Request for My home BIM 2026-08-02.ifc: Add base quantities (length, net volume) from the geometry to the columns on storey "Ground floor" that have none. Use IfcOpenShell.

First a look at what the model holds.

```python
import ifcopenshell
import ifcopenshell.util.element
import ifcopenshell.util.unit

model = ifcopenshell.open("My home BIM 2026-08-02.ifc")
print(model.schema)
for unit_type in ("LENGTHUNIT", "AREAUNIT", "VOLUMEUNIT"):
    print(unit_type, ifcopenshell.util.unit.calculate_unit_scale(model, unit_type))
storey = next(s for s in model.by_type("IfcBuildingStorey") if s.Name == "Ground floor")
columns = [e for e in ifcopenshell.util.element.get_decomposition(storey) if e.is_a("IfcColumn")]
for e in sorted(columns, key=lambda e: e.id()):
    print(e.id(), e.is_a(), e.Name, list(ifcopenshell.util.element.get_psets(e, qtos_only=True)), sep=" | ")
```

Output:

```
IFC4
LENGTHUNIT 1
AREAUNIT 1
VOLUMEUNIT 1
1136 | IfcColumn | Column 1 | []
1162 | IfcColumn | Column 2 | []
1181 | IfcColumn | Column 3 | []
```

```python
import ifcopenshell
import ifcopenshell.api.pset
import ifcopenshell.geom
import ifcopenshell.util.element
import ifcopenshell.util.shape
import ifcopenshell.util.unit

model = ifcopenshell.open("My home BIM 2026-08-02.ifc")
unit_scale = ifcopenshell.util.unit.calculate_unit_scale(model)
volume_scale = ifcopenshell.util.unit.calculate_unit_scale(model, "VOLUMEUNIT")
settings = ifcopenshell.geom.settings()

storey = next(s for s in model.by_type("IfcBuildingStorey") if s.Name == "Ground floor")
columns = [e for e in ifcopenshell.util.element.get_decomposition(storey) if e.is_a("IfcColumn")]

for e in sorted(columns, key=lambda e: e.id()):
    if ifcopenshell.util.element.get_psets(e, qtos_only=True, should_inherit=False):
        continue
    # Geometry comes back in metres, in the element's own axes.
    shape = ifcopenshell.geom.create_shape(settings, e)
    values = {
        "Length": ifcopenshell.util.shape.get_z(shape.geometry) / unit_scale,
        "NetVolume": ifcopenshell.util.shape.get_volume(shape.geometry) / volume_scale,
    }
    qto = ifcopenshell.api.pset.add_qto(model, product=e, name="Qto_ColumnBaseQuantities")
    ifcopenshell.api.pset.edit_qto(model, qto=qto, properties=values)
    print(e.id(), {k: round(v, 3) for k, v in values.items()})

model.write("My home BIM 2026-08-02_edited.ifc")
```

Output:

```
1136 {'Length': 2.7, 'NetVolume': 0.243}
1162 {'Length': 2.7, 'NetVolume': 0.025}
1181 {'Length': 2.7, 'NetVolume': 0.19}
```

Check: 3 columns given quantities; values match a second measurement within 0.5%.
